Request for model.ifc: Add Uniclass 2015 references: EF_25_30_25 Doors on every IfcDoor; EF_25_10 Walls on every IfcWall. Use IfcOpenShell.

First a look at what the model holds.

```python
import ifcopenshell

model = ifcopenshell.open("model.ifc")
print(model.schema)
print("classifications:", [c.Name for c in model.by_type("IfcClassification")])
for ifc_class in ("IfcDoor", "IfcRoof", "IfcStair", "IfcWall", "IfcWindow"):
    print(ifc_class, len(model.by_type(ifc_class)))
```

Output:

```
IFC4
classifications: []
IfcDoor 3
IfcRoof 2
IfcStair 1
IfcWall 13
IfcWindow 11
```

```python
import ifcopenshell
import ifcopenshell.api.classification

model = ifcopenshell.open("model.ifc")

system = ifcopenshell.api.classification.add_classification(model, classification="Uniclass 2015")

codes = {
    "IfcDoor": ("EF_25_30_25", "Doors"),
    "IfcWall": ("EF_25_10", "Walls"),
}
for ifc_class, (code, name) in codes.items():
    products = model.by_type(ifc_class)
    ifcopenshell.api.classification.add_reference(
        model, products=products, classification=system, identification=code, name=name
    )
    print(code, len(products))

model.write("model_updated.ifc")
```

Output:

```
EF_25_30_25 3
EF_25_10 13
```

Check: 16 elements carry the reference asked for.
